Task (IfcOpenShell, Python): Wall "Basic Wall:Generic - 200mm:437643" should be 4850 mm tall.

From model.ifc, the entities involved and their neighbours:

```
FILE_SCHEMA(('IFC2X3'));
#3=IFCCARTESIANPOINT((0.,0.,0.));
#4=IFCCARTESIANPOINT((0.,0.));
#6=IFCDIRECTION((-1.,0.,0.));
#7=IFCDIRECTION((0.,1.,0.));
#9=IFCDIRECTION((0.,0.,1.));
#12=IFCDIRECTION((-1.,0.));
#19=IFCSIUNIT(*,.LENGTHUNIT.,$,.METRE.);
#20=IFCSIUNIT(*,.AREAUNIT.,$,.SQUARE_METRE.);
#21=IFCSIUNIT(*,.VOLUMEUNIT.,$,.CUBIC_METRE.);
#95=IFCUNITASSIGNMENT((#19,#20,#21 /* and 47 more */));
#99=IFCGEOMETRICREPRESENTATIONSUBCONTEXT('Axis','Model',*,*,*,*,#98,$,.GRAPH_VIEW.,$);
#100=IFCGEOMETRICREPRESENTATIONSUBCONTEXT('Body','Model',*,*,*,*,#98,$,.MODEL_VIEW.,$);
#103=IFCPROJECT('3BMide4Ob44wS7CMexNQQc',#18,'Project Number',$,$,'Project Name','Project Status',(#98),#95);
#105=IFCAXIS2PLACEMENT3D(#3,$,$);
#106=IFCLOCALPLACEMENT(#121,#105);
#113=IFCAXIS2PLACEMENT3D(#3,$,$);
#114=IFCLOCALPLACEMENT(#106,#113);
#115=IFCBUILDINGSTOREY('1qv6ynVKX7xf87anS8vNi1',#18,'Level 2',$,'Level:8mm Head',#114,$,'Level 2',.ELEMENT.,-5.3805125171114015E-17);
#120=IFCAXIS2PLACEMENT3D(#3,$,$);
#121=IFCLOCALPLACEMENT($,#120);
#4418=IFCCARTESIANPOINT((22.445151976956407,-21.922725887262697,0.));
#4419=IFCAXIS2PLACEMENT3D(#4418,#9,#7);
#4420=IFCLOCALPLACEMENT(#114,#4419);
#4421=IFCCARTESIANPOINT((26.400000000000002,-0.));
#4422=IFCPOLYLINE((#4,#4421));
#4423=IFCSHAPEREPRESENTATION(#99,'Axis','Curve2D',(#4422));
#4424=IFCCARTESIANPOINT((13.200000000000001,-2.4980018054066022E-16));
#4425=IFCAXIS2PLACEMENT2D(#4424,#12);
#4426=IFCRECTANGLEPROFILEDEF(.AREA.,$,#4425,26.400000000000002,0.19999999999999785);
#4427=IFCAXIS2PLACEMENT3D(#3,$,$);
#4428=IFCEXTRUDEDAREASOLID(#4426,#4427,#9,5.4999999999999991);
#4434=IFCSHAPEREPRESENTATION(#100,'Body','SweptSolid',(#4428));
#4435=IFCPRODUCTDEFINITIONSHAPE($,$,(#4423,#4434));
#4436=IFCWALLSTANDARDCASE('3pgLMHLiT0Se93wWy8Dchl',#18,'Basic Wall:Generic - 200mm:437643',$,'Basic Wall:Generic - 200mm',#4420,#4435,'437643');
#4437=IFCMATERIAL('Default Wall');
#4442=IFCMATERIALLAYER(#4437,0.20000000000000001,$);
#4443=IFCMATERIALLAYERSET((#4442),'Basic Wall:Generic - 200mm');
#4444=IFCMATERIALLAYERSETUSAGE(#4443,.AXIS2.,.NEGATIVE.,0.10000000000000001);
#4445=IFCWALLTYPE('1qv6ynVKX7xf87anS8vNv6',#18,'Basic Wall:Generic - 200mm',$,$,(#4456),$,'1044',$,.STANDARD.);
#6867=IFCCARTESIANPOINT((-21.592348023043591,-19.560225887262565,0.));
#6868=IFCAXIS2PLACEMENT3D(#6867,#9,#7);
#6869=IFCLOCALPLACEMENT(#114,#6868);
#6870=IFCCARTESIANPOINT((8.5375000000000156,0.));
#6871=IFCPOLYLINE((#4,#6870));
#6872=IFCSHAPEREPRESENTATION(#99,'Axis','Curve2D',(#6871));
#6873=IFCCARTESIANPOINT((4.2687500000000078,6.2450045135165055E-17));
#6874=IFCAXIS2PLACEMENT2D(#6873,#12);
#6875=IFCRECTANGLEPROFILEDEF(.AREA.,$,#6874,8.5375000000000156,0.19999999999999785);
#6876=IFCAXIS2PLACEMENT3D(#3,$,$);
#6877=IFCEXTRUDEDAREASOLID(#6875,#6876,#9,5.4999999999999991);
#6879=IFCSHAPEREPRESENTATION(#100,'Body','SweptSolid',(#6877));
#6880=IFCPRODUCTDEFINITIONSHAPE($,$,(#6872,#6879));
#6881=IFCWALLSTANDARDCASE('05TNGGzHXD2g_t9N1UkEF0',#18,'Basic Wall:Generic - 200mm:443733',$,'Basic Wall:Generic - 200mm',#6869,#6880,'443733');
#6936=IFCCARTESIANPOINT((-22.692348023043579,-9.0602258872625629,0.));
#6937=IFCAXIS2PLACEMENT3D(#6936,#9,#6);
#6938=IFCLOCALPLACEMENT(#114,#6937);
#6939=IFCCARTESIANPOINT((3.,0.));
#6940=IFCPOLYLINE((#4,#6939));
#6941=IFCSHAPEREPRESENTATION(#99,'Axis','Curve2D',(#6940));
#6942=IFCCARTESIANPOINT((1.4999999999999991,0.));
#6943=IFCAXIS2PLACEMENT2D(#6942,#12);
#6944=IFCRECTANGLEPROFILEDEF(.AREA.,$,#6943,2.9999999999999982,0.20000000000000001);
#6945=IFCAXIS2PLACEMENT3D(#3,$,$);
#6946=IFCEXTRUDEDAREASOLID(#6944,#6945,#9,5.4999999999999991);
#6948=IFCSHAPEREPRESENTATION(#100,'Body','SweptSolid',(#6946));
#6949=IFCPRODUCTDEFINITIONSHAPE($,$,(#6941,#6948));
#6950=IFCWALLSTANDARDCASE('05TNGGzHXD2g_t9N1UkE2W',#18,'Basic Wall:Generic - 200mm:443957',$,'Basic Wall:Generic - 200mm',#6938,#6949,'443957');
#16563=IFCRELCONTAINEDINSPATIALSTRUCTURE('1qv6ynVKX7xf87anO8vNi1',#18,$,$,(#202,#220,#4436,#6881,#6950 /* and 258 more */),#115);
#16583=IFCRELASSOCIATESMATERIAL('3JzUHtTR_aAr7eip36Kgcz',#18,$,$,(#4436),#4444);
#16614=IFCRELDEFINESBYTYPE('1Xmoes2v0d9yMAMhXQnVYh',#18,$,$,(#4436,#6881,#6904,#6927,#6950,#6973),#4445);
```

```python
import ifcopenshell
import ifcopenshell.geom
import ifcopenshell.util.representation
import ifcopenshell.util.shape

model = ifcopenshell.open("model.ifc")
settings = ifcopenshell.geom.settings()


def volume(element):
    """Net volume in cubic metres, openings subtracted."""
    shape = ifcopenshell.geom.create_shape(settings, element)
    return ifcopenshell.util.shape.get_volume(shape.geometry)


wall = model.by_guid("3pgLMHLiT0Se93wWy8Dchl")
before = volume(wall)

body = ifcopenshell.util.representation.get_representation(wall, "Model", "Body")
solid = body.Items[0]
old_height = solid.Depth
solid.Depth = 4.85
after = volume(wall)

print(f"height {old_height:g} -> {solid.Depth:g}, volume {before:.3f} -> {after:.3f} m3")

model.write("model_rev.ifc")
```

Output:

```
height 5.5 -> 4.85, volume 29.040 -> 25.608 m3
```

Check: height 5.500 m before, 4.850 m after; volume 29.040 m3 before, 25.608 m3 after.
